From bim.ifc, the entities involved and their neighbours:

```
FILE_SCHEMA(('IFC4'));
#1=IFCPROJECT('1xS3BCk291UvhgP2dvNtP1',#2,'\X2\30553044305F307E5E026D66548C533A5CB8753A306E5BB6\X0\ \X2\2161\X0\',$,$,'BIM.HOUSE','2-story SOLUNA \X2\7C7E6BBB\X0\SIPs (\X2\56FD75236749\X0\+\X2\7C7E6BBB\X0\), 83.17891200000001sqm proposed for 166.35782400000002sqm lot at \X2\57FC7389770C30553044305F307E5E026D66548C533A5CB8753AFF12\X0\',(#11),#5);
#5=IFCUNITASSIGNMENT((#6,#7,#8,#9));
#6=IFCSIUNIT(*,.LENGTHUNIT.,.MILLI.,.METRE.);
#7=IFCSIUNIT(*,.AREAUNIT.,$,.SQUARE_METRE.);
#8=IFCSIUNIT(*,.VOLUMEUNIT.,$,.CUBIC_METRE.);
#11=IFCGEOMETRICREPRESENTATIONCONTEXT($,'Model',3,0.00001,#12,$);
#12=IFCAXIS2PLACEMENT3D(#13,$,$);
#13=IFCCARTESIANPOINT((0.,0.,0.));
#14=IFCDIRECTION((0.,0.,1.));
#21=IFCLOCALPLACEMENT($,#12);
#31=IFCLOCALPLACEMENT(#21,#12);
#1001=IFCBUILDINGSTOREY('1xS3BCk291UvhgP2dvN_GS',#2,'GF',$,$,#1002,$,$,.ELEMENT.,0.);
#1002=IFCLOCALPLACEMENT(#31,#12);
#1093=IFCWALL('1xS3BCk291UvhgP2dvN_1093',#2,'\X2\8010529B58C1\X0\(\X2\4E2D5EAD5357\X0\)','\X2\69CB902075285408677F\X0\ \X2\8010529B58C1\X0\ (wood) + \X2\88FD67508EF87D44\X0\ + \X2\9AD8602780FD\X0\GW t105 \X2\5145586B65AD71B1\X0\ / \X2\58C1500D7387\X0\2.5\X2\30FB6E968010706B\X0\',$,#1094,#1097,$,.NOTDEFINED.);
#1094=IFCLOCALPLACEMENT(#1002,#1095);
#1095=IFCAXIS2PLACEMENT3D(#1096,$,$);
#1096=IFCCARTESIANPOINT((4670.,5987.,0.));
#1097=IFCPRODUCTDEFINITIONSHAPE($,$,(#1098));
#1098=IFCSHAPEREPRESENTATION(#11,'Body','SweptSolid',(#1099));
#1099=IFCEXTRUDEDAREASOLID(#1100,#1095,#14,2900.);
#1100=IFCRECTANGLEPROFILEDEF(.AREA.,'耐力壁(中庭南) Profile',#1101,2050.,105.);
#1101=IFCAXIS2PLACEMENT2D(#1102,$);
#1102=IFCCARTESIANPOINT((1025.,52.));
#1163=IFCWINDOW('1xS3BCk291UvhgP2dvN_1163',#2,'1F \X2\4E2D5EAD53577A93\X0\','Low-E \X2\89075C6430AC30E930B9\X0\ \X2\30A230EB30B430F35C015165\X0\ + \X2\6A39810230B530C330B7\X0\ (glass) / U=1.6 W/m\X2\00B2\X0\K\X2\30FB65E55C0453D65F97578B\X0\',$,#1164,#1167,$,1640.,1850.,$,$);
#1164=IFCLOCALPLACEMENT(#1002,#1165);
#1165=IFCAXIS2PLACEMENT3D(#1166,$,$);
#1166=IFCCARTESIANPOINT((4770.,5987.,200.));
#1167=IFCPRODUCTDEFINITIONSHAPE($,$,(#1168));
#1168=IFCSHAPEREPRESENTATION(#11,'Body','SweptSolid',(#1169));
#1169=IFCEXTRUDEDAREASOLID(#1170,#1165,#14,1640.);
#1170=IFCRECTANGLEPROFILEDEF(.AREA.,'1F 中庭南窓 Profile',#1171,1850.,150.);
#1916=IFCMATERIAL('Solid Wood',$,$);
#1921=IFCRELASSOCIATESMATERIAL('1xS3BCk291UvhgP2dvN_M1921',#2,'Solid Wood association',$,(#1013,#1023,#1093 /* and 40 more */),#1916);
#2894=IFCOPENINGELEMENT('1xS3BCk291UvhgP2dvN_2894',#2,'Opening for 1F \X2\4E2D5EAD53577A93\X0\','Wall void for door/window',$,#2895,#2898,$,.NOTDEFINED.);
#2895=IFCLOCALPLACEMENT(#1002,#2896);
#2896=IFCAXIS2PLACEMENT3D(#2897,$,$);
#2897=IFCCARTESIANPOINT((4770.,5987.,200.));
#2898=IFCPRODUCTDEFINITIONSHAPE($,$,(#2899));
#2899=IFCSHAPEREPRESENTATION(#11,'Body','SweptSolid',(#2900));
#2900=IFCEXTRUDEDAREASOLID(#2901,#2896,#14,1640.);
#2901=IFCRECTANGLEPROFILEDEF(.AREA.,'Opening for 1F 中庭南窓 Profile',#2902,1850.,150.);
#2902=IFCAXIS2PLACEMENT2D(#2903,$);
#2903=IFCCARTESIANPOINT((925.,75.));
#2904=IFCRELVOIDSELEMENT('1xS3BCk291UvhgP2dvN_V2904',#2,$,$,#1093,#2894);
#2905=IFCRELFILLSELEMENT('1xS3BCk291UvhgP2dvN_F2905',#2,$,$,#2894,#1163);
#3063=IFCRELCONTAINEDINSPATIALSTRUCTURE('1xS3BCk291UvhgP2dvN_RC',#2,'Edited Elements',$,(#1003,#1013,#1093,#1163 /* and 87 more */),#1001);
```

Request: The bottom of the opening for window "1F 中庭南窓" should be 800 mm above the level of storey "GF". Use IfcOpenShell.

```python
import numpy as np
import ifcopenshell
import ifcopenshell.api.geometry
import ifcopenshell.geom
import ifcopenshell.util.element
import ifcopenshell.util.placement
import ifcopenshell.util.shape
import ifcopenshell.util.unit

model = ifcopenshell.open("bim.ifc")
unit_scale = ifcopenshell.util.unit.calculate_unit_scale(model)

window = model.by_guid("1xS3BCk291UvhgP2dvN_1163")
opening = window.FillsVoids[0].RelatingOpeningElement
storey = ifcopenshell.util.element.get_container(window, ifc_class="IfcBuildingStorey")
level = ifcopenshell.util.placement.get_local_placement(storey.ObjectPlacement)[2, 3]

# The opening's origin need not be at the sill, so measure its lowest point.
shape = ifcopenshell.geom.create_shape(ifcopenshell.geom.settings(), opening)
bottom = ifcopenshell.util.shape.get_shape_bottom_elevation(shape, shape.geometry) / unit_scale
dz = level + 800.0 - bottom

shift = np.array([0.0, 0.0, dz])
# The window is not placed relative to its opening, so move both.
for product in (opening, window):
    matrix = ifcopenshell.util.placement.get_local_placement(product.ObjectPlacement)
    matrix[:3, 3] += shift
    ifcopenshell.api.geometry.edit_object_placement(model, product=product, matrix=matrix, is_si=False)

print(f"moved by {dz * unit_scale:+.3f} m")

model.write("bim-out.ifc")
```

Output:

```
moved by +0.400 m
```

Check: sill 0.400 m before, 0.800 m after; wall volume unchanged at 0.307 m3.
